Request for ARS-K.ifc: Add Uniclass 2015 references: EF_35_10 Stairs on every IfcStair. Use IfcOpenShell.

First a look at what the model holds.

```python
import ifcopenshell

model = ifcopenshell.open("ARS-K.ifc")
print(model.schema)
print("classifications:", [c.Name for c in model.by_type("IfcClassification")])
for ifc_class in ("IfcDoor", "IfcRoof", "IfcStair", "IfcWall", "IfcWindow"):
    print(ifc_class, len(model.by_type(ifc_class)))
```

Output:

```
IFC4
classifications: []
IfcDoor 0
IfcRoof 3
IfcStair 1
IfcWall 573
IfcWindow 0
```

```python
import ifcopenshell
import ifcopenshell.api.classification

model = ifcopenshell.open("ARS-K.ifc")

system = ifcopenshell.api.classification.add_classification(model, classification="Uniclass 2015")

codes = {
    "IfcStair": ("EF_35_10", "Stairs"),
}
for ifc_class, (code, name) in codes.items():
    products = model.by_type(ifc_class)
    ifcopenshell.api.classification.add_reference(
        model, products=products, classification=system, identification=code, name=name
    )
    print(code, len(products))

model.write("ARS-K_rev.ifc")
```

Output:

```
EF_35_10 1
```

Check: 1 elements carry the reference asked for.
